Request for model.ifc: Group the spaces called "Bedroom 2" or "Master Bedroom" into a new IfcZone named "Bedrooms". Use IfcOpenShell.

First a look at what the model holds.

```python
import ifcopenshell

model = ifcopenshell.open("model.ifc")
print(model.schema)
seen = {}
for space in model.by_type("IfcSpace"):
    seen[space.LongName] = seen.get(space.LongName, 0) + 1
for name, count in sorted(seen.items(), key=str):
    print(count, "x", name)
print("zones:", [z.Name for z in model.by_type("IfcZone")][:20])
```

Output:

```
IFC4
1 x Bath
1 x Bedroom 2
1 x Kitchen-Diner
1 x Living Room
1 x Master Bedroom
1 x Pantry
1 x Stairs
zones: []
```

```python
import ifcopenshell
import ifcopenshell.api.group
import ifcopenshell.api.root

model = ifcopenshell.open("model.ifc")

names = {"Bedroom 2", "Master Bedroom"}
spaces = [s for s in model.by_type("IfcSpace") if s.LongName in names]

zone = ifcopenshell.api.root.create_entity(model, ifc_class="IfcZone", name="Bedrooms")
ifcopenshell.api.group.assign_group(model, products=spaces, group=zone)
print(len(spaces), "spaces in", zone.Name)

model.write("model_v2.ifc")
```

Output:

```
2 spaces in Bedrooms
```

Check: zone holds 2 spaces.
